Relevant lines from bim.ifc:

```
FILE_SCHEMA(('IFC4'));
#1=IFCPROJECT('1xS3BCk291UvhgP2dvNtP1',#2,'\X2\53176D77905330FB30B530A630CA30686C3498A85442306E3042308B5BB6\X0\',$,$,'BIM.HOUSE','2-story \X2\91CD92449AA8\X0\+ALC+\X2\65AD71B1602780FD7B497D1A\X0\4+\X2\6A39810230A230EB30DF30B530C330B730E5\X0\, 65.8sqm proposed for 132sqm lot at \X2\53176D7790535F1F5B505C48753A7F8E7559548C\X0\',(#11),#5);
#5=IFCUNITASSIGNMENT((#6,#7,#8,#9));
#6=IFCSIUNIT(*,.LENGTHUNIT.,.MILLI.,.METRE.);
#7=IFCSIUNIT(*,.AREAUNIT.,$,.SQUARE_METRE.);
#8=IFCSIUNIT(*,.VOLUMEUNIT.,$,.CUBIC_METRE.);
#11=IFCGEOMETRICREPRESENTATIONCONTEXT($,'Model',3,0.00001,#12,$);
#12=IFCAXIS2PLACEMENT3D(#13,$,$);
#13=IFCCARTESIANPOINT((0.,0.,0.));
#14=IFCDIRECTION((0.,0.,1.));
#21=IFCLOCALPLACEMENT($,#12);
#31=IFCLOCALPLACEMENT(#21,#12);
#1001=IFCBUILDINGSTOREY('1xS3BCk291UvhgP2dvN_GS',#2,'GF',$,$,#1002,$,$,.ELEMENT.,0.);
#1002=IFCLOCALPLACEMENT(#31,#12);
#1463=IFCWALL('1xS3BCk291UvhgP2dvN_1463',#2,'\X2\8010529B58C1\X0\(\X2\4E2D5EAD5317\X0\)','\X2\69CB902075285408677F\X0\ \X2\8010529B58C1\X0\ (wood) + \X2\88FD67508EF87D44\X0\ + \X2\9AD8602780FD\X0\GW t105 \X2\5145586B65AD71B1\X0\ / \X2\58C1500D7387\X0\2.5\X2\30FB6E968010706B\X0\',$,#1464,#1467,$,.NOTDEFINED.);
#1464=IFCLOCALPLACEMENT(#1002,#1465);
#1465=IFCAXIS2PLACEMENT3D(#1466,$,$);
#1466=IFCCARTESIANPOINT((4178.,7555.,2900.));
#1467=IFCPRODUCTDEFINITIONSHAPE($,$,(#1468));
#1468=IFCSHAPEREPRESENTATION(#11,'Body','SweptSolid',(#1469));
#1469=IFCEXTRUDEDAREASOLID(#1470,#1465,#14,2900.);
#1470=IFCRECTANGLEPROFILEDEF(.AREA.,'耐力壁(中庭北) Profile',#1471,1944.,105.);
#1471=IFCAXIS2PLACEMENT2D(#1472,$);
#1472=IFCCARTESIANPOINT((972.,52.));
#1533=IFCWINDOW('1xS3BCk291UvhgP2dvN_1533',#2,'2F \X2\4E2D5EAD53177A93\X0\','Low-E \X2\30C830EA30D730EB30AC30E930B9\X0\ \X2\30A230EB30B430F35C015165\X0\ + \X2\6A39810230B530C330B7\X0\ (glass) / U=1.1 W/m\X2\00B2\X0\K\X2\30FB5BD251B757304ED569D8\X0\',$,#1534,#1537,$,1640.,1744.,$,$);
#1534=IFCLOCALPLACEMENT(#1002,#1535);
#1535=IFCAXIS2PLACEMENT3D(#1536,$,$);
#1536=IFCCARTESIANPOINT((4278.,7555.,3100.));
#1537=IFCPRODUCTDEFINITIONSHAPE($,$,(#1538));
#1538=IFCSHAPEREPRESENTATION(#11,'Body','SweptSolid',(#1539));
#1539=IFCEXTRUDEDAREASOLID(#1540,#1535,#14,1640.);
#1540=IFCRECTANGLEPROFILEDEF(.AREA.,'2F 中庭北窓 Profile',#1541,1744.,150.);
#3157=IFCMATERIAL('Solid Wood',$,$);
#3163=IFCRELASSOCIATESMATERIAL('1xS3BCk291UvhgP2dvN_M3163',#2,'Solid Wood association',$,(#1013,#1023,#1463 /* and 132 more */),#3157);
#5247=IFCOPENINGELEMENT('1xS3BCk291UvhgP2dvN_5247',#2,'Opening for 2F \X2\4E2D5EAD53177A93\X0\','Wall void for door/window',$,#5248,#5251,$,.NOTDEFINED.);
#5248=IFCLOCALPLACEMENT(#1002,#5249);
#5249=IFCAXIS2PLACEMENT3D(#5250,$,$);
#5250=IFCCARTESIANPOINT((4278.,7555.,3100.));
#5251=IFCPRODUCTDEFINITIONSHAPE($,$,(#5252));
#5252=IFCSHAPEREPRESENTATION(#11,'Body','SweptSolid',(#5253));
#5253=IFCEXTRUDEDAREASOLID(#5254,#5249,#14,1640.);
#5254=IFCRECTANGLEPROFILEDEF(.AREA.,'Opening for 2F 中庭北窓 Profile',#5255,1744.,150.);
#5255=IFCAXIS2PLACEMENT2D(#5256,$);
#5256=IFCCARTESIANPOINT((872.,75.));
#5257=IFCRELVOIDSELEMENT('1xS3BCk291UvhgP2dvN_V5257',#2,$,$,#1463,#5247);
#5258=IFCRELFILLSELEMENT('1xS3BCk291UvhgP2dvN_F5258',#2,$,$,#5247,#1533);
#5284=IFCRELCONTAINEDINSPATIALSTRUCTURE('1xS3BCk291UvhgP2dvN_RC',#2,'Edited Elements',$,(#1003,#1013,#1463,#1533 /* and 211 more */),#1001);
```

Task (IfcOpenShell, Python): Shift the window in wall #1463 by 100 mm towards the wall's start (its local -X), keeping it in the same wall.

```python
import ifcopenshell
import ifcopenshell.api.geometry
import ifcopenshell.util.placement
import ifcopenshell.util.unit

model = ifcopenshell.open("bim.ifc")
unit_scale = ifcopenshell.util.unit.calculate_unit_scale(model)

window = model.by_id(1533)
opening = window.FillsVoids[0].RelatingOpeningElement
wall = opening.VoidsElements[0].RelatingBuildingElement

wall_matrix = ifcopenshell.util.placement.get_local_placement(wall.ObjectPlacement)
shift = wall_matrix[:3, 0] * -0.1 / unit_scale
before = ifcopenshell.util.placement.get_local_placement(window.ObjectPlacement)[:3, 3].copy()

# The window is not placed relative to its opening, so move both.
for product in (opening, window):
    matrix = ifcopenshell.util.placement.get_local_placement(product.ObjectPlacement)
    matrix[:3, 3] += shift
    ifcopenshell.api.geometry.edit_object_placement(model, product=product, matrix=matrix, is_si=False)

after = ifcopenshell.util.placement.get_local_placement(window.ObjectPlacement)[:3, 3]
print("window moved by", (after - before).round(3) + 0.0)

model.write("bim_v2.ifc")
```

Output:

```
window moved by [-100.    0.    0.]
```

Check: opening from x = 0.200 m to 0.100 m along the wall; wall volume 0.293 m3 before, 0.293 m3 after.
